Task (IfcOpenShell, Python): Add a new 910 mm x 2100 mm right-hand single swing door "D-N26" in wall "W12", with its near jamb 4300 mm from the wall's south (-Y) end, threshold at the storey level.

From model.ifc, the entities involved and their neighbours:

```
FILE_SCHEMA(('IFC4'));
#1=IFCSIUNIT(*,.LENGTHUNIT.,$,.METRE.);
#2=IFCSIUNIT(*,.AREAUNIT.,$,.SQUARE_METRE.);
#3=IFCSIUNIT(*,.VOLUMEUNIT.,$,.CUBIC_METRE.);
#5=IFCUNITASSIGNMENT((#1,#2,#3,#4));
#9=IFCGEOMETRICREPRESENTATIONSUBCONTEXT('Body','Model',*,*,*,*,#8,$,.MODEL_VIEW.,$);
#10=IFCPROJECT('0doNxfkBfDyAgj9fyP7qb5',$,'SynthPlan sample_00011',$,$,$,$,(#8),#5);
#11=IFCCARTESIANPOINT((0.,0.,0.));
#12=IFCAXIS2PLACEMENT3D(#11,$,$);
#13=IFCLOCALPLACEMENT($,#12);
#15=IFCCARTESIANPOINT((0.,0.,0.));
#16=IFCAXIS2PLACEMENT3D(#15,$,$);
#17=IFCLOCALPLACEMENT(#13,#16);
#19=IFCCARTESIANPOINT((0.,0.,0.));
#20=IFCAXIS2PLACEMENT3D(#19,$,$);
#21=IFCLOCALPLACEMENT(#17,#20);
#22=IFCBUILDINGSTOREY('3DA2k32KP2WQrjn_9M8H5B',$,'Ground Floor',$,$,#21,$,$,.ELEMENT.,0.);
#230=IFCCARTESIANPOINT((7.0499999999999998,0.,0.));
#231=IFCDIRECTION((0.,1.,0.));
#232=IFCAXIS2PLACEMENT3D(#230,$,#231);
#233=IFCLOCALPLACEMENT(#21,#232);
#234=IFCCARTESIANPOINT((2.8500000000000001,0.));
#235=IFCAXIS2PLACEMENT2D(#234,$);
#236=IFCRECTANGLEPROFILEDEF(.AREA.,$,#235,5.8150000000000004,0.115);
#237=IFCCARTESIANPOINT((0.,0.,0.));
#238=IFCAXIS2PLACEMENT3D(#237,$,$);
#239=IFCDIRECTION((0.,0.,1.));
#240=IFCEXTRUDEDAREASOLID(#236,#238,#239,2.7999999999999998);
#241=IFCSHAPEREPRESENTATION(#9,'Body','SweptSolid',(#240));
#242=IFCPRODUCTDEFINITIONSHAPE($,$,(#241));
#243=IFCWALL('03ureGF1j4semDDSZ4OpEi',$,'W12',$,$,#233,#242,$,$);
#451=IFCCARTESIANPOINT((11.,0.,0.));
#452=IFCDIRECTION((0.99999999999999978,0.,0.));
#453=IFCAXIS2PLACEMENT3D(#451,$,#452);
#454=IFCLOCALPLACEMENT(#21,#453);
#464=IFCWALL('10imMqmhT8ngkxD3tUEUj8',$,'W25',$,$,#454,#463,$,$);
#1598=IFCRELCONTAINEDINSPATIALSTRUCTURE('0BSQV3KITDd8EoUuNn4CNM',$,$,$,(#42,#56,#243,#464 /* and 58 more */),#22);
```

```python
import numpy as np
import ifcopenshell
import ifcopenshell.api.feature
import ifcopenshell.api.geometry
import ifcopenshell.api.root
import ifcopenshell.api.spatial
import ifcopenshell.geom
import ifcopenshell.util.element
import ifcopenshell.util.placement
import ifcopenshell.util.representation
import ifcopenshell.util.shape
import ifcopenshell.util.unit

model = ifcopenshell.open("model.ifc")
unit_scale = ifcopenshell.util.unit.calculate_unit_scale(model)
settings = ifcopenshell.geom.settings()


def volume(element):
    """Net volume in cubic metres, openings subtracted."""
    shape = ifcopenshell.geom.create_shape(settings, element)
    return ifcopenshell.util.shape.get_volume(shape.geometry)


wall = model.by_guid("03ureGF1j4semDDSZ4OpEi")
storey = ifcopenshell.util.element.get_container(wall, ifc_class="IfcBuildingStorey")
context = ifcopenshell.util.representation.get_context(model, "Model", "Body", "MODEL_VIEW")
before = volume(wall)

width, height, from_end, sill = 0.91, 2.1, 4.3, 0.0  # metres

# The wall runs along its own X axis, and the end named is its -X end.
wall_shape = ifcopenshell.geom.create_shape(settings, wall)
x, y, z = ifcopenshell.util.shape.get_vertices(wall_shape.geometry).T
start = x.min() + from_end
face, thickness = float(y.min()), float(y.max() - y.min())
wall_matrix = ifcopenshell.util.placement.get_local_placement(wall.ObjectPlacement)
level = ifcopenshell.util.placement.get_local_placement(storey.ObjectPlacement)[2, 3]


def in_wall(x, y):
    """Placement at x, y metres in the wall's axes, at sill height."""
    matrix = wall_matrix.copy()
    matrix[:, 3] = wall_matrix @ np.array([x / unit_scale, y / unit_scale, 0.0, 1.0])
    matrix[2, 3] = level + sill / unit_scale
    return matrix


# Opening: a box that overshoots both wall faces by 50 mm.
opening = ifcopenshell.api.root.create_entity(model, ifc_class="IfcOpeningElement", predefined_type="OPENING")
box = ifcopenshell.api.geometry.add_wall_representation(
    model, context=context, length=width, height=height, thickness=thickness + 0.1
)
ifcopenshell.api.geometry.assign_representation(model, product=opening, representation=box)
ifcopenshell.api.geometry.edit_object_placement(model, product=opening, matrix=in_wall(start, face - 0.05), is_si=False)
ifcopenshell.api.feature.add_feature(model, feature=opening, element=wall)

door = ifcopenshell.api.root.create_entity(model, ifc_class="IfcDoor", name="D-N26", predefined_type="DOOR")
door.OverallWidth, door.OverallHeight = width / unit_scale, height / unit_scale
door.OperationType = "SINGLE_SWING_RIGHT"
body = ifcopenshell.api.geometry.add_door_representation(
    model,
    context=context,
    overall_width=door.OverallWidth,
    overall_height=door.OverallHeight,
    operation_type="SINGLE_SWING_RIGHT",
    lining_properties={"LiningDepth": thickness / unit_scale, "ThresholdDepth": thickness / unit_scale},
)
ifcopenshell.api.geometry.assign_representation(model, product=door, representation=body)
ifcopenshell.api.spatial.assign_container(model, products=[door], relating_structure=storey)
ifcopenshell.api.feature.add_filling(model, opening=opening, element=door)

# The lining spans the wall, so the door starts at the wall face.
ifcopenshell.api.geometry.edit_object_placement(model, product=door, matrix=in_wall(start, face), is_si=False)

after = volume(wall)

print(f"wall volume {before:.3f} -> {after:.3f} m3")

model.write("model_updated.ifc")
```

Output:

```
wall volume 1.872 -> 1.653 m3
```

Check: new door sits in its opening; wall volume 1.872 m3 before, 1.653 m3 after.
